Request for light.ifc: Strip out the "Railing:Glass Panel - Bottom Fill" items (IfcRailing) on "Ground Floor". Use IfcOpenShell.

First a look at what the model holds.

```python
import ifcopenshell
import ifcopenshell.util.element

model = ifcopenshell.open("light.ifc")
print(model.schema)
storey = next(s for s in model.by_type("IfcBuildingStorey") if s.Name == "Ground Floor")
railings = [e for e in ifcopenshell.util.element.get_decomposition(storey) if e.is_a("IfcRailing")]
seen = {}
for e in railings:
    element_type = ifcopenshell.util.element.get_type(e)
    name = element_type.Name if element_type not in (None, e) else None
    seen[name] = seen.get(name, 0) + 1
for name, count in sorted(seen.items(), key=str):
    print(count, "x", name)
```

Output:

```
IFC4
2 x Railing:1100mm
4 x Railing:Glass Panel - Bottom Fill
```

```python
import ifcopenshell
import ifcopenshell.api.root
import ifcopenshell.util.element

model = ifcopenshell.open("light.ifc")

storey = next(s for s in model.by_type("IfcBuildingStorey") if s.Name == "Ground Floor")
railings = [e for e in ifcopenshell.util.element.get_decomposition(storey) if e.is_a("IfcRailing")]
targets = [e for e in railings if (t := ifcopenshell.util.element.get_type(e)) not in (None, e) and t.Name == "Railing:Glass Panel - Bottom Fill"]

for e in targets:
    ifcopenshell.api.root.remove_product(model, product=e)
print(len(targets), "removed")

model.write("light-out.ifc")
```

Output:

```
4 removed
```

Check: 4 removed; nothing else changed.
